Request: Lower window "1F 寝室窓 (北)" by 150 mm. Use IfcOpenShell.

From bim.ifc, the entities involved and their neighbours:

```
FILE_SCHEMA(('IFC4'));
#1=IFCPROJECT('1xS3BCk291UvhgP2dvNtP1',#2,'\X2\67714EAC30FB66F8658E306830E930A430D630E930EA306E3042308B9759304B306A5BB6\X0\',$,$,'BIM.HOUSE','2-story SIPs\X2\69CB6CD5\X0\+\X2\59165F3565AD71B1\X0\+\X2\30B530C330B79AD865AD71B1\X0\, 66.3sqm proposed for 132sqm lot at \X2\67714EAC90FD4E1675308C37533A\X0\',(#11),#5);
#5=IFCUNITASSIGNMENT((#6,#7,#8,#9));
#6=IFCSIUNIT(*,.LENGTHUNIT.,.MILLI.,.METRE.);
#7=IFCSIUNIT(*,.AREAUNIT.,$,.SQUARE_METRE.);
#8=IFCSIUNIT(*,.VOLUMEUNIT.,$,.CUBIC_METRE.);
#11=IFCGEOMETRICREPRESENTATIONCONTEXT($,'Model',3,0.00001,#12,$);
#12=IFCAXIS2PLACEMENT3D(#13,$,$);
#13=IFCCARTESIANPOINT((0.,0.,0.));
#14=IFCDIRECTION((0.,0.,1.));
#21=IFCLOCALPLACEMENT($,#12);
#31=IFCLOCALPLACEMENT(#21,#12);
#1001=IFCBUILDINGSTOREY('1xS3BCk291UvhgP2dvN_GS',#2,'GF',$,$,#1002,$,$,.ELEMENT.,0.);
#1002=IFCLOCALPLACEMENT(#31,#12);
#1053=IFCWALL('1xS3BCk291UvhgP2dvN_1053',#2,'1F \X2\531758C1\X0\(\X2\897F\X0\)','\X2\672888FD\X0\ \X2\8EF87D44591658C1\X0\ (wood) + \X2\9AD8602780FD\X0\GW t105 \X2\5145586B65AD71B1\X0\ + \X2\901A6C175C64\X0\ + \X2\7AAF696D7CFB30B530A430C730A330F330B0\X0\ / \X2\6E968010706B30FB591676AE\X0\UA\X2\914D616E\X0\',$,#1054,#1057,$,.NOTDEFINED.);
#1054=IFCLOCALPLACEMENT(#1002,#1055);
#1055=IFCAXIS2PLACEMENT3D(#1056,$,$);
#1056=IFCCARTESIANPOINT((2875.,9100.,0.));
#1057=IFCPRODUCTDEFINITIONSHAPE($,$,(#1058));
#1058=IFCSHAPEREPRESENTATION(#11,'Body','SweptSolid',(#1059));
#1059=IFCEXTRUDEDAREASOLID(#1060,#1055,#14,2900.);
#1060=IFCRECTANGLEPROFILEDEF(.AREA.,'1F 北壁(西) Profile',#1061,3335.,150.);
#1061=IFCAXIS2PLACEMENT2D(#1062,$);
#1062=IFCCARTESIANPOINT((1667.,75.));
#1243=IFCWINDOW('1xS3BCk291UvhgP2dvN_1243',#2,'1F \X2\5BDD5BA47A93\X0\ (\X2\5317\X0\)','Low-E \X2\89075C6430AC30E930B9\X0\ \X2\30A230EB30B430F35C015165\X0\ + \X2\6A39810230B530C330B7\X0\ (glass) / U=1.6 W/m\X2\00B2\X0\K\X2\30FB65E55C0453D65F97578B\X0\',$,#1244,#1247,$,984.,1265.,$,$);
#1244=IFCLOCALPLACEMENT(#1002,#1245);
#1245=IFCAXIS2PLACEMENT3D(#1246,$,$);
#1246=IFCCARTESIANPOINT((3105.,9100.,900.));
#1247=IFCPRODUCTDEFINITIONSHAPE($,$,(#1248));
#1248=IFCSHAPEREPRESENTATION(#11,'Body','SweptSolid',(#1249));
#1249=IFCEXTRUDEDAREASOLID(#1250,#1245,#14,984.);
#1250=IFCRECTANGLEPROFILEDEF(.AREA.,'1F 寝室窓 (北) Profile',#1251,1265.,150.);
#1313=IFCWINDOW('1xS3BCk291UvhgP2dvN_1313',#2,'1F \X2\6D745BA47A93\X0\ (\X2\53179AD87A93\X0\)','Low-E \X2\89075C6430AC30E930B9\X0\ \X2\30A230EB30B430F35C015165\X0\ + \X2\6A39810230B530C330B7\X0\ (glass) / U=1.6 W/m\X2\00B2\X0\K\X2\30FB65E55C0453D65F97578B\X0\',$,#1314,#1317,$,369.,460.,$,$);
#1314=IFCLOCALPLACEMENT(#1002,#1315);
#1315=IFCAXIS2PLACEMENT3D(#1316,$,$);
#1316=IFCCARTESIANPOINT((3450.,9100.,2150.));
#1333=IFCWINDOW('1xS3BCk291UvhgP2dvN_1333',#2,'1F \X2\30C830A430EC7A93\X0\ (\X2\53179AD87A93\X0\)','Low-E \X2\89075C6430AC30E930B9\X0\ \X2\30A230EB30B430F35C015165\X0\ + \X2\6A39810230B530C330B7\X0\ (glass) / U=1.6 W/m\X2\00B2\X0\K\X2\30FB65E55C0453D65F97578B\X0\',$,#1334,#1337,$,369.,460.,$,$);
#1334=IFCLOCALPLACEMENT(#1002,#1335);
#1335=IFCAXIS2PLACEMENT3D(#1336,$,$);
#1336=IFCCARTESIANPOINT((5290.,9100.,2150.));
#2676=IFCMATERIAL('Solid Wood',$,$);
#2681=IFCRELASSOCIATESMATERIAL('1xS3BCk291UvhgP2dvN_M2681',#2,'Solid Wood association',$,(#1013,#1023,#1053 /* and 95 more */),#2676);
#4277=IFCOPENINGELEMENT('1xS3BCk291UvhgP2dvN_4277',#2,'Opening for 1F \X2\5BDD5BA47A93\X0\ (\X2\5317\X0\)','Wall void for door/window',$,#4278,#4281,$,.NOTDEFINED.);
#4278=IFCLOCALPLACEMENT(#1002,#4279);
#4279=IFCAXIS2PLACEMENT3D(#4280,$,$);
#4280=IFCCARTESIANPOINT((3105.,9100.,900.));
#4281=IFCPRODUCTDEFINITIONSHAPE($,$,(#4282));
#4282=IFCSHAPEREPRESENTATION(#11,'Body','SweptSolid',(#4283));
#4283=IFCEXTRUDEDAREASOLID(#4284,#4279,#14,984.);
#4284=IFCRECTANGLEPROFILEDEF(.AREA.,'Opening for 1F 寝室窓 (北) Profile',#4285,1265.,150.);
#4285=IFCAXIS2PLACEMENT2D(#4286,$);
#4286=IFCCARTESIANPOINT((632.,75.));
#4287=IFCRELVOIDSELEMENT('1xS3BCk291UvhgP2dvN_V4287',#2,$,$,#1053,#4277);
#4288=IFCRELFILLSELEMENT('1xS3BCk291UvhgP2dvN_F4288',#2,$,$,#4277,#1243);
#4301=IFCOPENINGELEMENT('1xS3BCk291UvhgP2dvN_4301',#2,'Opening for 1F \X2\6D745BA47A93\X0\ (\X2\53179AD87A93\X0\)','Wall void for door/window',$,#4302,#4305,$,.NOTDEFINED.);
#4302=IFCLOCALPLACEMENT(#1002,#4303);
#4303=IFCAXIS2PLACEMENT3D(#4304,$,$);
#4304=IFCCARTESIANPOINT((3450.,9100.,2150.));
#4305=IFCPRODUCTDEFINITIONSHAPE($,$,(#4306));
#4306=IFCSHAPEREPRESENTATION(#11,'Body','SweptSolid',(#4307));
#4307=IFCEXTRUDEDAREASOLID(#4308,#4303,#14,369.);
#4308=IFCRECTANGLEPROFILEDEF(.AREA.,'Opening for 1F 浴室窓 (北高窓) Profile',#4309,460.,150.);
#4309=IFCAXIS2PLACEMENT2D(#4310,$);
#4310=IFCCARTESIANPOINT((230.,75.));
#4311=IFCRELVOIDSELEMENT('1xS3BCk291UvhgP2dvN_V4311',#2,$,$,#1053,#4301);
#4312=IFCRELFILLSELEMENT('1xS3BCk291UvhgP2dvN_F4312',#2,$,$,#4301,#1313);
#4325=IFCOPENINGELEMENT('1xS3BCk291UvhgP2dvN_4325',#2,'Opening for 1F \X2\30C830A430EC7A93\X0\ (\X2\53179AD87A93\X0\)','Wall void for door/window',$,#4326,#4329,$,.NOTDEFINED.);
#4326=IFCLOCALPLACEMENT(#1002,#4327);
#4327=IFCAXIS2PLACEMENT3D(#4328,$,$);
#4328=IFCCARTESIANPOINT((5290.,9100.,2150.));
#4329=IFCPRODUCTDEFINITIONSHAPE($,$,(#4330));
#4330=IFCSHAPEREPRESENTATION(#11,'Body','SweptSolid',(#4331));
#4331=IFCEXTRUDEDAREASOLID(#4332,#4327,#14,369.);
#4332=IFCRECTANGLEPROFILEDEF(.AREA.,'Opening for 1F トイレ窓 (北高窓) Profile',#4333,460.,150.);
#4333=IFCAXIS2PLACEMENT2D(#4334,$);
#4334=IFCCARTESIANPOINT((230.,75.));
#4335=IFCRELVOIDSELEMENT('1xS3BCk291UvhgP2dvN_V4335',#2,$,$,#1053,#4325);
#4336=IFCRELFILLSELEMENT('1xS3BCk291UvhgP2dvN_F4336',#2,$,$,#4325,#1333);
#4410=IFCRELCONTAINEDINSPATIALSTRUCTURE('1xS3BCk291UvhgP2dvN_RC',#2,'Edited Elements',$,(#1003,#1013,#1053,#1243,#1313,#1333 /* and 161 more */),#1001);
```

```python
import numpy as np
import ifcopenshell
import ifcopenshell.api.geometry
import ifcopenshell.util.placement
import ifcopenshell.util.unit

model = ifcopenshell.open("bim.ifc")
unit_scale = ifcopenshell.util.unit.calculate_unit_scale(model)

window = model.by_guid("1xS3BCk291UvhgP2dvN_1243")
opening = window.FillsVoids[0].RelatingOpeningElement
dz = -0.15 / unit_scale

shift = np.array([0.0, 0.0, dz])
# The window is not placed relative to its opening, so move both.
for product in (opening, window):
    matrix = ifcopenshell.util.placement.get_local_placement(product.ObjectPlacement)
    matrix[:3, 3] += shift
    ifcopenshell.api.geometry.edit_object_placement(model, product=product, matrix=matrix, is_si=False)

print(f"moved by {dz * unit_scale:+.3f} m")

model.write("bim_edited.ifc")
```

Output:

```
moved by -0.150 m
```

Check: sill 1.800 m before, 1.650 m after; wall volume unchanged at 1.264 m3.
